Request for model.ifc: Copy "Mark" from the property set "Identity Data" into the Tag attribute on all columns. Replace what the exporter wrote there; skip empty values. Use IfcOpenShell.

First a look at what the model holds.

```python
import ifcopenshell
import ifcopenshell.util.element

model = ifcopenshell.open("model.ifc")
print(model.schema)
columns = model.by_type("IfcColumn")
print(len(columns), "columns")
for e in columns[:8]:
    source = ifcopenshell.util.element.get_pset(e, "Identity Data", "Mark")
    target = e.Tag
    print(e.id(), repr(source), repr(target), sep=" | ")
```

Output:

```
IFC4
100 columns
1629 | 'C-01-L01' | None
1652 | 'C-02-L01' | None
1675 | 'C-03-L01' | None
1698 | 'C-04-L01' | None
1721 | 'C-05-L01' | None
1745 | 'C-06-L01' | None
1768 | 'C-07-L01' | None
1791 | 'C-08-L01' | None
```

```python
import ifcopenshell
import ifcopenshell.util.element

model = ifcopenshell.open("model.ifc")

count = 0
for e in model.by_type("IfcColumn"):
    value = ifcopenshell.util.element.get_pset(e, "Identity Data", "Mark")
    current = e.Tag
    if not value or not value.strip() or current == value:
        continue
    e.Tag = value
    count += 1

print(count, "columns updated")

model.write("model_updated.ifc")
```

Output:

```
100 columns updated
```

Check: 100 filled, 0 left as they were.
